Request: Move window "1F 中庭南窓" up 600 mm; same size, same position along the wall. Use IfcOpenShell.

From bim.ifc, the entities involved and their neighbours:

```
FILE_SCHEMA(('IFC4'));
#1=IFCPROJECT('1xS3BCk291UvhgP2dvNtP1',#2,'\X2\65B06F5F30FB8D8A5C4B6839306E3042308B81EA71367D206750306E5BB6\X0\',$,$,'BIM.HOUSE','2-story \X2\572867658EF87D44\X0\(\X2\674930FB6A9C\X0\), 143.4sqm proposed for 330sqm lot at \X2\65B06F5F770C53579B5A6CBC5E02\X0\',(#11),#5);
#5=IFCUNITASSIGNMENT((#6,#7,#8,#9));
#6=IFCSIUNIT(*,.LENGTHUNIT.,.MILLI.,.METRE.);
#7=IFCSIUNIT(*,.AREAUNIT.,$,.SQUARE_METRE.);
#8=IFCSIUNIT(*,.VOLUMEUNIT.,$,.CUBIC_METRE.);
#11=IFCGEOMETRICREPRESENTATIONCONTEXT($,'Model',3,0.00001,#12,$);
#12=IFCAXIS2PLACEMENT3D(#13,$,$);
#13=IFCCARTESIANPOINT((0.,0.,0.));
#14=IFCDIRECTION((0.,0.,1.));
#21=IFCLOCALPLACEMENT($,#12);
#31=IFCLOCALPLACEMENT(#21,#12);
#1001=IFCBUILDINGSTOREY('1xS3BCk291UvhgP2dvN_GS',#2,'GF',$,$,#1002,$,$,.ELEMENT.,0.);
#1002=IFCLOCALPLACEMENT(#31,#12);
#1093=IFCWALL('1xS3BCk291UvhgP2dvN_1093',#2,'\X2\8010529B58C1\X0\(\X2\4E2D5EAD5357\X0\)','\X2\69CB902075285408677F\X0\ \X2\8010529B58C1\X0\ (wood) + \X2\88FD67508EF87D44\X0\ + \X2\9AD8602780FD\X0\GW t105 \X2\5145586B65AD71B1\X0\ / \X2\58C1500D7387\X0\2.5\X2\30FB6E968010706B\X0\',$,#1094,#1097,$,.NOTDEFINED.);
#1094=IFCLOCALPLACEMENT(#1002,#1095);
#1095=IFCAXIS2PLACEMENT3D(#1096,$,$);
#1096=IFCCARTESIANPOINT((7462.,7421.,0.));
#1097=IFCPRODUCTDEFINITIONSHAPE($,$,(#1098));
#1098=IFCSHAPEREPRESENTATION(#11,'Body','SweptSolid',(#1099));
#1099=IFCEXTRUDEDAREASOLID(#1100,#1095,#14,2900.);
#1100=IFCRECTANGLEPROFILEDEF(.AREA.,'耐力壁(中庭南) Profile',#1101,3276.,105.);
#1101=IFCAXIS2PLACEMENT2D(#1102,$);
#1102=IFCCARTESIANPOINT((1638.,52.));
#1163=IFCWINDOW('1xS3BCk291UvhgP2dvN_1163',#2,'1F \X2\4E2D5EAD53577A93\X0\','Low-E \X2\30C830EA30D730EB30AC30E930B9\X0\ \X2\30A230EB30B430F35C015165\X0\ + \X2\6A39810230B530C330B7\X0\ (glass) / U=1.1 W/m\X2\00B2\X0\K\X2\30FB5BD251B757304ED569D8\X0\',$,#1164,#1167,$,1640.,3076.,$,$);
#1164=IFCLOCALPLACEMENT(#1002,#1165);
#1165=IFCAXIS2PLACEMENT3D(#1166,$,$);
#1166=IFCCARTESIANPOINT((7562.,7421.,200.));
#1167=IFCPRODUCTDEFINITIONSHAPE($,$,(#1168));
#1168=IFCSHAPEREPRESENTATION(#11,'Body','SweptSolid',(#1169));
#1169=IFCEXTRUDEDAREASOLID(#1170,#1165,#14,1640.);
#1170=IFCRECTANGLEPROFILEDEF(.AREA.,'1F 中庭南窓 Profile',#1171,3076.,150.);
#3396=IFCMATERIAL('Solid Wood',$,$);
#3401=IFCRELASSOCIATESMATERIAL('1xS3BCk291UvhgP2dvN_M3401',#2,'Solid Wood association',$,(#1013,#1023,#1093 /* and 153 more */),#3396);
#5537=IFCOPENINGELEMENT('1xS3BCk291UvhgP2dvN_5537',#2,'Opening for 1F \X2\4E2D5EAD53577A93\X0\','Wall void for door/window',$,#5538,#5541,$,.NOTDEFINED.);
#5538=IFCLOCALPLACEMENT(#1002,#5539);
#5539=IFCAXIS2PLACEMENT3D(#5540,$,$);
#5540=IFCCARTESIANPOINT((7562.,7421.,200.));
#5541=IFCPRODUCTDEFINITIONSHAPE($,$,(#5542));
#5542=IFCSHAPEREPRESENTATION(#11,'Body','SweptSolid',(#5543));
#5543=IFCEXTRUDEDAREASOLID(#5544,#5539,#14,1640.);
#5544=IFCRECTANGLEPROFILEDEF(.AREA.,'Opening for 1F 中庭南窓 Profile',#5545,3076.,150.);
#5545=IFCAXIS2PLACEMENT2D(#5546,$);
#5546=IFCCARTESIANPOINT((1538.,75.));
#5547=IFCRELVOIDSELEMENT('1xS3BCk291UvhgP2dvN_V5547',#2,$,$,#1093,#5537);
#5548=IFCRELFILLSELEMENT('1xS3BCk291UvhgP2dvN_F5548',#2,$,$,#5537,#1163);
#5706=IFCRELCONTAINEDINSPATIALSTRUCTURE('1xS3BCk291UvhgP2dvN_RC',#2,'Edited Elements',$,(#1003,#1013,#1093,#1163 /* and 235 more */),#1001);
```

```python
import numpy as np
import ifcopenshell
import ifcopenshell.api.geometry
import ifcopenshell.util.placement
import ifcopenshell.util.unit

model = ifcopenshell.open("bim.ifc")
unit_scale = ifcopenshell.util.unit.calculate_unit_scale(model)

window = model.by_guid("1xS3BCk291UvhgP2dvN_1163")
opening = window.FillsVoids[0].RelatingOpeningElement
dz = 600.0

shift = np.array([0.0, 0.0, dz])
# The window is not placed relative to its opening, so move both.
for product in (opening, window):
    matrix = ifcopenshell.util.placement.get_local_placement(product.ObjectPlacement)
    matrix[:3, 3] += shift
    ifcopenshell.api.geometry.edit_object_placement(model, product=product, matrix=matrix, is_si=False)

print(f"moved by {dz * unit_scale:+.3f} m")

model.write("bim_edited.ifc")
```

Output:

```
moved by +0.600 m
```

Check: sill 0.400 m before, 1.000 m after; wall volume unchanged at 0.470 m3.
